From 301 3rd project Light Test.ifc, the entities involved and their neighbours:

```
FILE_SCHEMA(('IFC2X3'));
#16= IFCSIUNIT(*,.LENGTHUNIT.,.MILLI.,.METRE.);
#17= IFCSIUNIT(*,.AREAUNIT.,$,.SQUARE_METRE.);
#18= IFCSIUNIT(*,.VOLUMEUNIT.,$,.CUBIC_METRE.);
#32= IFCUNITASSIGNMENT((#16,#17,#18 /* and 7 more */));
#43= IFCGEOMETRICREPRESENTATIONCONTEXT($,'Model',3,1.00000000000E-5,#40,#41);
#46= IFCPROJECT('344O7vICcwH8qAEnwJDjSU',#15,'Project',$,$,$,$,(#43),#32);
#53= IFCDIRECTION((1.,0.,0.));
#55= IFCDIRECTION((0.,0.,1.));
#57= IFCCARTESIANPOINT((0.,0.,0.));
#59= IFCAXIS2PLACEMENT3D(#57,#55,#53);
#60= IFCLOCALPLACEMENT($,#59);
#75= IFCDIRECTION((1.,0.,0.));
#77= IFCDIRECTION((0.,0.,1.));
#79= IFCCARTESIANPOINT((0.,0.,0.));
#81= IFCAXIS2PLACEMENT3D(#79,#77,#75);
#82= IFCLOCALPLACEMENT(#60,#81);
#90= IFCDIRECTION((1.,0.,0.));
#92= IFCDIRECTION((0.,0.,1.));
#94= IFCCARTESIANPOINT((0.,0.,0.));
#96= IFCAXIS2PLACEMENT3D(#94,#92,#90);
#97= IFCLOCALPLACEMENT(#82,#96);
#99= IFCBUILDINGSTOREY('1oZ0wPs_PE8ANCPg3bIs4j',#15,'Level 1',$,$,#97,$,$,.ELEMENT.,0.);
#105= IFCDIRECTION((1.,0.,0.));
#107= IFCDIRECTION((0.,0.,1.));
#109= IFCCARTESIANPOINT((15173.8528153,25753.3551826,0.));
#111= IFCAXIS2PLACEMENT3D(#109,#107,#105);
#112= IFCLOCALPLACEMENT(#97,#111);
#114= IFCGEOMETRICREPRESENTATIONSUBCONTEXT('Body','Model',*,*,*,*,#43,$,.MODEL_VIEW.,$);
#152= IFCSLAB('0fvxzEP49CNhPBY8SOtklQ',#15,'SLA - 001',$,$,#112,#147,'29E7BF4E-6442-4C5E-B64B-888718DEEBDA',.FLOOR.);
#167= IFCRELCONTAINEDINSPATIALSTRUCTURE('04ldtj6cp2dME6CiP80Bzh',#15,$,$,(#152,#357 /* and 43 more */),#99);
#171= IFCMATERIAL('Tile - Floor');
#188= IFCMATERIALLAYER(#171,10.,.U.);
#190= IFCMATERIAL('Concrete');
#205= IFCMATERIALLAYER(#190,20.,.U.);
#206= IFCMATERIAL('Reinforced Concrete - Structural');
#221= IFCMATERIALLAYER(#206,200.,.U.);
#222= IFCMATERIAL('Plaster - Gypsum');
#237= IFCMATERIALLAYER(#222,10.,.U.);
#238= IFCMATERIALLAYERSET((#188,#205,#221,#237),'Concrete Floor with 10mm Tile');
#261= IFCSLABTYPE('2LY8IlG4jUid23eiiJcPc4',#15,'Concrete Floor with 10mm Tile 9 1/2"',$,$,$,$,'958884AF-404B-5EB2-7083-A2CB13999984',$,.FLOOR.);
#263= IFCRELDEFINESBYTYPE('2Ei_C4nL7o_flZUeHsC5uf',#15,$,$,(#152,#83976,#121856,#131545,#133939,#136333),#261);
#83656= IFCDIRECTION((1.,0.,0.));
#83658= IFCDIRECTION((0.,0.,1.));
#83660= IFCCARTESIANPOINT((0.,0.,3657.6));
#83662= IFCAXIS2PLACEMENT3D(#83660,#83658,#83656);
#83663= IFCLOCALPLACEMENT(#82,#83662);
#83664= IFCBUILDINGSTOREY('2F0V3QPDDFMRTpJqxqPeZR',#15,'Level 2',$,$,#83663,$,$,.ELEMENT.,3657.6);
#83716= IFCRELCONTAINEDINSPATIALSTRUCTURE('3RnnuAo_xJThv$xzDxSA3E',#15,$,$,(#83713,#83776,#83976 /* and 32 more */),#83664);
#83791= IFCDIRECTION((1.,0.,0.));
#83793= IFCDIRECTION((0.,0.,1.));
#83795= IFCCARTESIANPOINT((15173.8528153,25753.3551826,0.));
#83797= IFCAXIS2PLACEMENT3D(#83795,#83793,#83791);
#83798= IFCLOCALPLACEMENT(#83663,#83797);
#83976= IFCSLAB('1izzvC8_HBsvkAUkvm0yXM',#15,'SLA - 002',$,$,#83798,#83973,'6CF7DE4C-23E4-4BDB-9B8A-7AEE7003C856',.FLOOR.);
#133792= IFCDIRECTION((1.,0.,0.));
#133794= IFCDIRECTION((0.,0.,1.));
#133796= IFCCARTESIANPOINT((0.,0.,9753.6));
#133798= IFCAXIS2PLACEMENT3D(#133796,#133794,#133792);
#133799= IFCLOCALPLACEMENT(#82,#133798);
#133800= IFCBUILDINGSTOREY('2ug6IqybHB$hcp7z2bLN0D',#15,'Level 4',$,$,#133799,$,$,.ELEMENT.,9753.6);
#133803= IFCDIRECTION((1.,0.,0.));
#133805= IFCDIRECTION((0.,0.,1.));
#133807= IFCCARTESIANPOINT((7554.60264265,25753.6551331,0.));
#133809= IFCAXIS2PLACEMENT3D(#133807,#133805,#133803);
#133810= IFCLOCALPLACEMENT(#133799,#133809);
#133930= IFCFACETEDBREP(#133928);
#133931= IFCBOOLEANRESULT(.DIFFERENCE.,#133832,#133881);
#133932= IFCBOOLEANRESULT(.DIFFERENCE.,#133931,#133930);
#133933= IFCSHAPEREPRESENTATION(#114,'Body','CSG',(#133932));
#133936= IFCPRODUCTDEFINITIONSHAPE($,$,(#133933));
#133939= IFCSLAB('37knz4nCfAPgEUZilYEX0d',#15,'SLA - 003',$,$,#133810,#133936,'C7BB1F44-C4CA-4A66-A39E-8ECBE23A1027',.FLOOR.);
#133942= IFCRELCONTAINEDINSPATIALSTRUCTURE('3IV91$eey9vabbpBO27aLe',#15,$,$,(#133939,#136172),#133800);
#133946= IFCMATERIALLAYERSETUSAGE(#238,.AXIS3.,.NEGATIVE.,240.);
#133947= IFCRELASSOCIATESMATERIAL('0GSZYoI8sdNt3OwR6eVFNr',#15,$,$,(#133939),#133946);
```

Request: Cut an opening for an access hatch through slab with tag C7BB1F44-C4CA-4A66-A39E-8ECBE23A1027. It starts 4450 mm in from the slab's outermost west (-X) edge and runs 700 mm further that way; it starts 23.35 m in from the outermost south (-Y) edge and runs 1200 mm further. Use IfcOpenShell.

```python
import numpy as np
import ifcopenshell
import ifcopenshell.api.feature
import ifcopenshell.api.geometry
import ifcopenshell.api.root
import ifcopenshell.geom
import ifcopenshell.util.placement
import ifcopenshell.util.representation
import ifcopenshell.util.shape
import ifcopenshell.util.unit

model = ifcopenshell.open("301 3rd project Light Test.ifc")
unit_scale = ifcopenshell.util.unit.calculate_unit_scale(model)
settings = ifcopenshell.geom.settings()


def volume(element):
    """Net volume in cubic metres, openings subtracted."""
    shape = ifcopenshell.geom.create_shape(settings, element)
    return ifcopenshell.util.shape.get_volume(shape.geometry)


slab = model.by_guid("37knz4nCfAPgEUZilYEX0d")
before = volume(slab)

# Extent in the slab's own axes, in metres. The edges named are its -X and -Y sides.
slab_shape = ifcopenshell.geom.create_shape(settings, slab)
vertices = ifcopenshell.util.shape.get_vertices(slab_shape.geometry)
x_min, y_min, bottom = vertices.min(axis=0)
top = vertices[:, 2].max()

opening = ifcopenshell.api.root.create_entity(model, ifc_class="IfcOpeningElement", name="Access hatch opening")
context = ifcopenshell.util.representation.get_context(model, "Model", "Body", "MODEL_VIEW")
width, depth = 0.7, 1.2
outline = [(0.0, 0.0), (width, 0.0), (width, depth), (0.0, depth), (0.0, 0.0)]
# Overshoot both faces by 50 mm so the cut is clean.
shape = ifcopenshell.api.geometry.add_slab_representation(
    model, context=context, depth=top - bottom + 0.1, polyline=outline
)
ifcopenshell.api.geometry.assign_representation(model, product=opening, representation=shape)

matrix = ifcopenshell.util.placement.get_local_placement(slab.ObjectPlacement)
matrix[:, 3] = matrix @ np.append(np.array([x_min + 4.45, y_min + 23.35, bottom - 0.05]) / unit_scale, 1.0)
ifcopenshell.api.geometry.edit_object_placement(model, product=opening, matrix=matrix, is_si=False)
ifcopenshell.api.feature.add_feature(model, feature=opening, element=slab)

after = volume(slab)

print(f"slab volume {before:.3f} -> {after:.3f} m3")

model.write("301 3rd project Light Test_v2.ifc")
```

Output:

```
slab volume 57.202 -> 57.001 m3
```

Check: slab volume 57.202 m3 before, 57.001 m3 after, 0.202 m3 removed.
